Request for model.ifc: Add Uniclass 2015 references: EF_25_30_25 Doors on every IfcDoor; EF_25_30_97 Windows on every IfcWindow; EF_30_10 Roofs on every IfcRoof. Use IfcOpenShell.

First a look at what the model holds.

```python
import ifcopenshell

model = ifcopenshell.open("model.ifc")
print(model.schema)
print("classifications:", [c.Name for c in model.by_type("IfcClassification")])
for ifc_class in ("IfcDoor", "IfcRoof", "IfcStair", "IfcWall", "IfcWindow"):
    print(ifc_class, len(model.by_type(ifc_class)))
```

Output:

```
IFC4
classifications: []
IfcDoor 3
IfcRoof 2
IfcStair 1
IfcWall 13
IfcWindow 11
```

```python
import ifcopenshell
import ifcopenshell.api.classification

model = ifcopenshell.open("model.ifc")

system = ifcopenshell.api.classification.add_classification(model, classification="Uniclass 2015")

codes = {
    "IfcDoor": ("EF_25_30_25", "Doors"),
    "IfcWindow": ("EF_25_30_97", "Windows"),
    "IfcRoof": ("EF_30_10", "Roofs"),
}
for ifc_class, (code, name) in codes.items():
    products = model.by_type(ifc_class)
    ifcopenshell.api.classification.add_reference(
        model, products=products, classification=system, identification=code, name=name
    )
    print(code, len(products))

model.write("model_edited.ifc")
```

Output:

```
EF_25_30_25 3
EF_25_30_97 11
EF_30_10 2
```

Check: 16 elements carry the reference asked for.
